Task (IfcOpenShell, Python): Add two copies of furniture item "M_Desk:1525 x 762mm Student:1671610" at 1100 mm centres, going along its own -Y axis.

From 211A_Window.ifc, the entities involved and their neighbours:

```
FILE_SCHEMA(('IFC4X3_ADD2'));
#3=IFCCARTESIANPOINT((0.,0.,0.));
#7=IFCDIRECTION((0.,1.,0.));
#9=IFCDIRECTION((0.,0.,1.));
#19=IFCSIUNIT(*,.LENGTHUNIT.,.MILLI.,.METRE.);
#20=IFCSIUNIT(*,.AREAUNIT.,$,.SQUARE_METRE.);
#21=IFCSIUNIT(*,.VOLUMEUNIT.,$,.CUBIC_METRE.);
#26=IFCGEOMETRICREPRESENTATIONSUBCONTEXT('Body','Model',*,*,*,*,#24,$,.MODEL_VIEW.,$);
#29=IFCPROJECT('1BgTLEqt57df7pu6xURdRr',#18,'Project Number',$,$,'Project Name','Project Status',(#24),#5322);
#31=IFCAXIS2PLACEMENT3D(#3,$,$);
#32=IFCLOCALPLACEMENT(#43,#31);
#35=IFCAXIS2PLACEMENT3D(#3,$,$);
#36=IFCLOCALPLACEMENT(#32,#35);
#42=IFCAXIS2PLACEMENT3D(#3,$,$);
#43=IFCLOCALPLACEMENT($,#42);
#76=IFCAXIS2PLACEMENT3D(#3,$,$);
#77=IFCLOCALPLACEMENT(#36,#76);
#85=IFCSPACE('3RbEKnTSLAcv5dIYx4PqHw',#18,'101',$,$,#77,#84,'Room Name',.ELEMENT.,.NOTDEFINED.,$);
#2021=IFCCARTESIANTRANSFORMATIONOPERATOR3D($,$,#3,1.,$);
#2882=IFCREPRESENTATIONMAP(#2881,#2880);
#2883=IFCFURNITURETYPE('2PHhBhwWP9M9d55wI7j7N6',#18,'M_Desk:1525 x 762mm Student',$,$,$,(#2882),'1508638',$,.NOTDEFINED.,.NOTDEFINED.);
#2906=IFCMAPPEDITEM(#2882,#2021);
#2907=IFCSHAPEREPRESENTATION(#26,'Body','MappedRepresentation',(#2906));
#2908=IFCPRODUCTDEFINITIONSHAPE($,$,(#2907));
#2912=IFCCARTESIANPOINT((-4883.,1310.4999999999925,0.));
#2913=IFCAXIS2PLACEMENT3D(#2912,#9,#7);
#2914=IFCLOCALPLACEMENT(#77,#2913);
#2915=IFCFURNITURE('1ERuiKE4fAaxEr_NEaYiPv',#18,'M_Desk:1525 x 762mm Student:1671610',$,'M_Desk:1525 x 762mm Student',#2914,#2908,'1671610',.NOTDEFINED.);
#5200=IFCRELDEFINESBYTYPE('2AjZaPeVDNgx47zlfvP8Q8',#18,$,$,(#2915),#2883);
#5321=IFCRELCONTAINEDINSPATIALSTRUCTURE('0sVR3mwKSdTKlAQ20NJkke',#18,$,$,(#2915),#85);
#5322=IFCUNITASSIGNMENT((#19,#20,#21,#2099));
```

```python
import ifcopenshell
import ifcopenshell.api.geometry
import ifcopenshell.api.root
import ifcopenshell.util.element
import ifcopenshell.util.placement

model = ifcopenshell.open("211A_Window.ifc")


def reuse_history(source, copy):
    """copy_class also copies each property set's owner history, people and application; keep the originals."""
    for rel in copy.IsDefinedBy:
        if rel.is_a("IfcRelDefinesByProperties") and (history := rel.RelatingPropertyDefinition.OwnerHistory):
            rel.RelatingPropertyDefinition.OwnerHistory = source.OwnerHistory
            ifcopenshell.util.element.remove_deep2(model, history)


source = model.by_guid("1ERuiKE4fAaxEr_NEaYiPv")
base = ifcopenshell.util.placement.get_local_placement(source.ObjectPlacement)
step = -base[:3, 1] * 1100.0

for i in range(1, 3):
    copy = ifcopenshell.api.root.copy_class(model, product=source)
    copy.Representation = ifcopenshell.util.element.copy_deep(
        model, source.Representation, exclude=["IfcGeometricRepresentationContext", "IfcRepresentationMap"]
    )
    copy.Name = "M_Desk:1525 x 762mm Student"
    copy.Tag = None
    reuse_history(source, copy)
    matrix = base.copy()
    matrix[:3, 3] += i * step
    print("added at", matrix[:3, 3].round(3) + 0.0)
    ifcopenshell.api.geometry.edit_object_placement(model, product=copy, matrix=matrix, is_si=False)

model.write("211A_Window_rev.ifc")
```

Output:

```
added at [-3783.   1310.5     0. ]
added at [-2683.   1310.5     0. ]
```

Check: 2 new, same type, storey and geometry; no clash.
